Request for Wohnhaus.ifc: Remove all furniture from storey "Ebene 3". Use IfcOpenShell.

First a look at what the model holds.

```python
import ifcopenshell
import ifcopenshell.util.element

model = ifcopenshell.open("Wohnhaus.ifc")
print(model.schema)
storey = next(s for s in model.by_type("IfcBuildingStorey") if s.Name == "Ebene 3")
furniture = [e for e in ifcopenshell.util.element.get_decomposition(storey) if e.is_a("IfcFurnishingElement")]
seen = {}
for e in furniture:
    element_type = ifcopenshell.util.element.get_type(e)
    name = element_type.Name if element_type not in (None, e) else None
    seen[name] = seen.get(name, 0) + 1
for name, count in sorted(seen.items(), key=str):
    print(count, "x", name)
```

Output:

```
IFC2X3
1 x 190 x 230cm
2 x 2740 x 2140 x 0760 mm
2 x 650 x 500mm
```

```python
import ifcopenshell
import ifcopenshell.api.root
import ifcopenshell.util.element

model = ifcopenshell.open("Wohnhaus.ifc")

storey = next(s for s in model.by_type("IfcBuildingStorey") if s.Name == "Ebene 3")
furniture = [e for e in ifcopenshell.util.element.get_decomposition(storey) if e.is_a("IfcFurnishingElement")]

for e in furniture:
    ifcopenshell.api.root.remove_product(model, product=e)
print(len(furniture), "removed")

model.write("Wohnhaus_edited.ifc")
```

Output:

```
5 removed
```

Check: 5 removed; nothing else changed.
